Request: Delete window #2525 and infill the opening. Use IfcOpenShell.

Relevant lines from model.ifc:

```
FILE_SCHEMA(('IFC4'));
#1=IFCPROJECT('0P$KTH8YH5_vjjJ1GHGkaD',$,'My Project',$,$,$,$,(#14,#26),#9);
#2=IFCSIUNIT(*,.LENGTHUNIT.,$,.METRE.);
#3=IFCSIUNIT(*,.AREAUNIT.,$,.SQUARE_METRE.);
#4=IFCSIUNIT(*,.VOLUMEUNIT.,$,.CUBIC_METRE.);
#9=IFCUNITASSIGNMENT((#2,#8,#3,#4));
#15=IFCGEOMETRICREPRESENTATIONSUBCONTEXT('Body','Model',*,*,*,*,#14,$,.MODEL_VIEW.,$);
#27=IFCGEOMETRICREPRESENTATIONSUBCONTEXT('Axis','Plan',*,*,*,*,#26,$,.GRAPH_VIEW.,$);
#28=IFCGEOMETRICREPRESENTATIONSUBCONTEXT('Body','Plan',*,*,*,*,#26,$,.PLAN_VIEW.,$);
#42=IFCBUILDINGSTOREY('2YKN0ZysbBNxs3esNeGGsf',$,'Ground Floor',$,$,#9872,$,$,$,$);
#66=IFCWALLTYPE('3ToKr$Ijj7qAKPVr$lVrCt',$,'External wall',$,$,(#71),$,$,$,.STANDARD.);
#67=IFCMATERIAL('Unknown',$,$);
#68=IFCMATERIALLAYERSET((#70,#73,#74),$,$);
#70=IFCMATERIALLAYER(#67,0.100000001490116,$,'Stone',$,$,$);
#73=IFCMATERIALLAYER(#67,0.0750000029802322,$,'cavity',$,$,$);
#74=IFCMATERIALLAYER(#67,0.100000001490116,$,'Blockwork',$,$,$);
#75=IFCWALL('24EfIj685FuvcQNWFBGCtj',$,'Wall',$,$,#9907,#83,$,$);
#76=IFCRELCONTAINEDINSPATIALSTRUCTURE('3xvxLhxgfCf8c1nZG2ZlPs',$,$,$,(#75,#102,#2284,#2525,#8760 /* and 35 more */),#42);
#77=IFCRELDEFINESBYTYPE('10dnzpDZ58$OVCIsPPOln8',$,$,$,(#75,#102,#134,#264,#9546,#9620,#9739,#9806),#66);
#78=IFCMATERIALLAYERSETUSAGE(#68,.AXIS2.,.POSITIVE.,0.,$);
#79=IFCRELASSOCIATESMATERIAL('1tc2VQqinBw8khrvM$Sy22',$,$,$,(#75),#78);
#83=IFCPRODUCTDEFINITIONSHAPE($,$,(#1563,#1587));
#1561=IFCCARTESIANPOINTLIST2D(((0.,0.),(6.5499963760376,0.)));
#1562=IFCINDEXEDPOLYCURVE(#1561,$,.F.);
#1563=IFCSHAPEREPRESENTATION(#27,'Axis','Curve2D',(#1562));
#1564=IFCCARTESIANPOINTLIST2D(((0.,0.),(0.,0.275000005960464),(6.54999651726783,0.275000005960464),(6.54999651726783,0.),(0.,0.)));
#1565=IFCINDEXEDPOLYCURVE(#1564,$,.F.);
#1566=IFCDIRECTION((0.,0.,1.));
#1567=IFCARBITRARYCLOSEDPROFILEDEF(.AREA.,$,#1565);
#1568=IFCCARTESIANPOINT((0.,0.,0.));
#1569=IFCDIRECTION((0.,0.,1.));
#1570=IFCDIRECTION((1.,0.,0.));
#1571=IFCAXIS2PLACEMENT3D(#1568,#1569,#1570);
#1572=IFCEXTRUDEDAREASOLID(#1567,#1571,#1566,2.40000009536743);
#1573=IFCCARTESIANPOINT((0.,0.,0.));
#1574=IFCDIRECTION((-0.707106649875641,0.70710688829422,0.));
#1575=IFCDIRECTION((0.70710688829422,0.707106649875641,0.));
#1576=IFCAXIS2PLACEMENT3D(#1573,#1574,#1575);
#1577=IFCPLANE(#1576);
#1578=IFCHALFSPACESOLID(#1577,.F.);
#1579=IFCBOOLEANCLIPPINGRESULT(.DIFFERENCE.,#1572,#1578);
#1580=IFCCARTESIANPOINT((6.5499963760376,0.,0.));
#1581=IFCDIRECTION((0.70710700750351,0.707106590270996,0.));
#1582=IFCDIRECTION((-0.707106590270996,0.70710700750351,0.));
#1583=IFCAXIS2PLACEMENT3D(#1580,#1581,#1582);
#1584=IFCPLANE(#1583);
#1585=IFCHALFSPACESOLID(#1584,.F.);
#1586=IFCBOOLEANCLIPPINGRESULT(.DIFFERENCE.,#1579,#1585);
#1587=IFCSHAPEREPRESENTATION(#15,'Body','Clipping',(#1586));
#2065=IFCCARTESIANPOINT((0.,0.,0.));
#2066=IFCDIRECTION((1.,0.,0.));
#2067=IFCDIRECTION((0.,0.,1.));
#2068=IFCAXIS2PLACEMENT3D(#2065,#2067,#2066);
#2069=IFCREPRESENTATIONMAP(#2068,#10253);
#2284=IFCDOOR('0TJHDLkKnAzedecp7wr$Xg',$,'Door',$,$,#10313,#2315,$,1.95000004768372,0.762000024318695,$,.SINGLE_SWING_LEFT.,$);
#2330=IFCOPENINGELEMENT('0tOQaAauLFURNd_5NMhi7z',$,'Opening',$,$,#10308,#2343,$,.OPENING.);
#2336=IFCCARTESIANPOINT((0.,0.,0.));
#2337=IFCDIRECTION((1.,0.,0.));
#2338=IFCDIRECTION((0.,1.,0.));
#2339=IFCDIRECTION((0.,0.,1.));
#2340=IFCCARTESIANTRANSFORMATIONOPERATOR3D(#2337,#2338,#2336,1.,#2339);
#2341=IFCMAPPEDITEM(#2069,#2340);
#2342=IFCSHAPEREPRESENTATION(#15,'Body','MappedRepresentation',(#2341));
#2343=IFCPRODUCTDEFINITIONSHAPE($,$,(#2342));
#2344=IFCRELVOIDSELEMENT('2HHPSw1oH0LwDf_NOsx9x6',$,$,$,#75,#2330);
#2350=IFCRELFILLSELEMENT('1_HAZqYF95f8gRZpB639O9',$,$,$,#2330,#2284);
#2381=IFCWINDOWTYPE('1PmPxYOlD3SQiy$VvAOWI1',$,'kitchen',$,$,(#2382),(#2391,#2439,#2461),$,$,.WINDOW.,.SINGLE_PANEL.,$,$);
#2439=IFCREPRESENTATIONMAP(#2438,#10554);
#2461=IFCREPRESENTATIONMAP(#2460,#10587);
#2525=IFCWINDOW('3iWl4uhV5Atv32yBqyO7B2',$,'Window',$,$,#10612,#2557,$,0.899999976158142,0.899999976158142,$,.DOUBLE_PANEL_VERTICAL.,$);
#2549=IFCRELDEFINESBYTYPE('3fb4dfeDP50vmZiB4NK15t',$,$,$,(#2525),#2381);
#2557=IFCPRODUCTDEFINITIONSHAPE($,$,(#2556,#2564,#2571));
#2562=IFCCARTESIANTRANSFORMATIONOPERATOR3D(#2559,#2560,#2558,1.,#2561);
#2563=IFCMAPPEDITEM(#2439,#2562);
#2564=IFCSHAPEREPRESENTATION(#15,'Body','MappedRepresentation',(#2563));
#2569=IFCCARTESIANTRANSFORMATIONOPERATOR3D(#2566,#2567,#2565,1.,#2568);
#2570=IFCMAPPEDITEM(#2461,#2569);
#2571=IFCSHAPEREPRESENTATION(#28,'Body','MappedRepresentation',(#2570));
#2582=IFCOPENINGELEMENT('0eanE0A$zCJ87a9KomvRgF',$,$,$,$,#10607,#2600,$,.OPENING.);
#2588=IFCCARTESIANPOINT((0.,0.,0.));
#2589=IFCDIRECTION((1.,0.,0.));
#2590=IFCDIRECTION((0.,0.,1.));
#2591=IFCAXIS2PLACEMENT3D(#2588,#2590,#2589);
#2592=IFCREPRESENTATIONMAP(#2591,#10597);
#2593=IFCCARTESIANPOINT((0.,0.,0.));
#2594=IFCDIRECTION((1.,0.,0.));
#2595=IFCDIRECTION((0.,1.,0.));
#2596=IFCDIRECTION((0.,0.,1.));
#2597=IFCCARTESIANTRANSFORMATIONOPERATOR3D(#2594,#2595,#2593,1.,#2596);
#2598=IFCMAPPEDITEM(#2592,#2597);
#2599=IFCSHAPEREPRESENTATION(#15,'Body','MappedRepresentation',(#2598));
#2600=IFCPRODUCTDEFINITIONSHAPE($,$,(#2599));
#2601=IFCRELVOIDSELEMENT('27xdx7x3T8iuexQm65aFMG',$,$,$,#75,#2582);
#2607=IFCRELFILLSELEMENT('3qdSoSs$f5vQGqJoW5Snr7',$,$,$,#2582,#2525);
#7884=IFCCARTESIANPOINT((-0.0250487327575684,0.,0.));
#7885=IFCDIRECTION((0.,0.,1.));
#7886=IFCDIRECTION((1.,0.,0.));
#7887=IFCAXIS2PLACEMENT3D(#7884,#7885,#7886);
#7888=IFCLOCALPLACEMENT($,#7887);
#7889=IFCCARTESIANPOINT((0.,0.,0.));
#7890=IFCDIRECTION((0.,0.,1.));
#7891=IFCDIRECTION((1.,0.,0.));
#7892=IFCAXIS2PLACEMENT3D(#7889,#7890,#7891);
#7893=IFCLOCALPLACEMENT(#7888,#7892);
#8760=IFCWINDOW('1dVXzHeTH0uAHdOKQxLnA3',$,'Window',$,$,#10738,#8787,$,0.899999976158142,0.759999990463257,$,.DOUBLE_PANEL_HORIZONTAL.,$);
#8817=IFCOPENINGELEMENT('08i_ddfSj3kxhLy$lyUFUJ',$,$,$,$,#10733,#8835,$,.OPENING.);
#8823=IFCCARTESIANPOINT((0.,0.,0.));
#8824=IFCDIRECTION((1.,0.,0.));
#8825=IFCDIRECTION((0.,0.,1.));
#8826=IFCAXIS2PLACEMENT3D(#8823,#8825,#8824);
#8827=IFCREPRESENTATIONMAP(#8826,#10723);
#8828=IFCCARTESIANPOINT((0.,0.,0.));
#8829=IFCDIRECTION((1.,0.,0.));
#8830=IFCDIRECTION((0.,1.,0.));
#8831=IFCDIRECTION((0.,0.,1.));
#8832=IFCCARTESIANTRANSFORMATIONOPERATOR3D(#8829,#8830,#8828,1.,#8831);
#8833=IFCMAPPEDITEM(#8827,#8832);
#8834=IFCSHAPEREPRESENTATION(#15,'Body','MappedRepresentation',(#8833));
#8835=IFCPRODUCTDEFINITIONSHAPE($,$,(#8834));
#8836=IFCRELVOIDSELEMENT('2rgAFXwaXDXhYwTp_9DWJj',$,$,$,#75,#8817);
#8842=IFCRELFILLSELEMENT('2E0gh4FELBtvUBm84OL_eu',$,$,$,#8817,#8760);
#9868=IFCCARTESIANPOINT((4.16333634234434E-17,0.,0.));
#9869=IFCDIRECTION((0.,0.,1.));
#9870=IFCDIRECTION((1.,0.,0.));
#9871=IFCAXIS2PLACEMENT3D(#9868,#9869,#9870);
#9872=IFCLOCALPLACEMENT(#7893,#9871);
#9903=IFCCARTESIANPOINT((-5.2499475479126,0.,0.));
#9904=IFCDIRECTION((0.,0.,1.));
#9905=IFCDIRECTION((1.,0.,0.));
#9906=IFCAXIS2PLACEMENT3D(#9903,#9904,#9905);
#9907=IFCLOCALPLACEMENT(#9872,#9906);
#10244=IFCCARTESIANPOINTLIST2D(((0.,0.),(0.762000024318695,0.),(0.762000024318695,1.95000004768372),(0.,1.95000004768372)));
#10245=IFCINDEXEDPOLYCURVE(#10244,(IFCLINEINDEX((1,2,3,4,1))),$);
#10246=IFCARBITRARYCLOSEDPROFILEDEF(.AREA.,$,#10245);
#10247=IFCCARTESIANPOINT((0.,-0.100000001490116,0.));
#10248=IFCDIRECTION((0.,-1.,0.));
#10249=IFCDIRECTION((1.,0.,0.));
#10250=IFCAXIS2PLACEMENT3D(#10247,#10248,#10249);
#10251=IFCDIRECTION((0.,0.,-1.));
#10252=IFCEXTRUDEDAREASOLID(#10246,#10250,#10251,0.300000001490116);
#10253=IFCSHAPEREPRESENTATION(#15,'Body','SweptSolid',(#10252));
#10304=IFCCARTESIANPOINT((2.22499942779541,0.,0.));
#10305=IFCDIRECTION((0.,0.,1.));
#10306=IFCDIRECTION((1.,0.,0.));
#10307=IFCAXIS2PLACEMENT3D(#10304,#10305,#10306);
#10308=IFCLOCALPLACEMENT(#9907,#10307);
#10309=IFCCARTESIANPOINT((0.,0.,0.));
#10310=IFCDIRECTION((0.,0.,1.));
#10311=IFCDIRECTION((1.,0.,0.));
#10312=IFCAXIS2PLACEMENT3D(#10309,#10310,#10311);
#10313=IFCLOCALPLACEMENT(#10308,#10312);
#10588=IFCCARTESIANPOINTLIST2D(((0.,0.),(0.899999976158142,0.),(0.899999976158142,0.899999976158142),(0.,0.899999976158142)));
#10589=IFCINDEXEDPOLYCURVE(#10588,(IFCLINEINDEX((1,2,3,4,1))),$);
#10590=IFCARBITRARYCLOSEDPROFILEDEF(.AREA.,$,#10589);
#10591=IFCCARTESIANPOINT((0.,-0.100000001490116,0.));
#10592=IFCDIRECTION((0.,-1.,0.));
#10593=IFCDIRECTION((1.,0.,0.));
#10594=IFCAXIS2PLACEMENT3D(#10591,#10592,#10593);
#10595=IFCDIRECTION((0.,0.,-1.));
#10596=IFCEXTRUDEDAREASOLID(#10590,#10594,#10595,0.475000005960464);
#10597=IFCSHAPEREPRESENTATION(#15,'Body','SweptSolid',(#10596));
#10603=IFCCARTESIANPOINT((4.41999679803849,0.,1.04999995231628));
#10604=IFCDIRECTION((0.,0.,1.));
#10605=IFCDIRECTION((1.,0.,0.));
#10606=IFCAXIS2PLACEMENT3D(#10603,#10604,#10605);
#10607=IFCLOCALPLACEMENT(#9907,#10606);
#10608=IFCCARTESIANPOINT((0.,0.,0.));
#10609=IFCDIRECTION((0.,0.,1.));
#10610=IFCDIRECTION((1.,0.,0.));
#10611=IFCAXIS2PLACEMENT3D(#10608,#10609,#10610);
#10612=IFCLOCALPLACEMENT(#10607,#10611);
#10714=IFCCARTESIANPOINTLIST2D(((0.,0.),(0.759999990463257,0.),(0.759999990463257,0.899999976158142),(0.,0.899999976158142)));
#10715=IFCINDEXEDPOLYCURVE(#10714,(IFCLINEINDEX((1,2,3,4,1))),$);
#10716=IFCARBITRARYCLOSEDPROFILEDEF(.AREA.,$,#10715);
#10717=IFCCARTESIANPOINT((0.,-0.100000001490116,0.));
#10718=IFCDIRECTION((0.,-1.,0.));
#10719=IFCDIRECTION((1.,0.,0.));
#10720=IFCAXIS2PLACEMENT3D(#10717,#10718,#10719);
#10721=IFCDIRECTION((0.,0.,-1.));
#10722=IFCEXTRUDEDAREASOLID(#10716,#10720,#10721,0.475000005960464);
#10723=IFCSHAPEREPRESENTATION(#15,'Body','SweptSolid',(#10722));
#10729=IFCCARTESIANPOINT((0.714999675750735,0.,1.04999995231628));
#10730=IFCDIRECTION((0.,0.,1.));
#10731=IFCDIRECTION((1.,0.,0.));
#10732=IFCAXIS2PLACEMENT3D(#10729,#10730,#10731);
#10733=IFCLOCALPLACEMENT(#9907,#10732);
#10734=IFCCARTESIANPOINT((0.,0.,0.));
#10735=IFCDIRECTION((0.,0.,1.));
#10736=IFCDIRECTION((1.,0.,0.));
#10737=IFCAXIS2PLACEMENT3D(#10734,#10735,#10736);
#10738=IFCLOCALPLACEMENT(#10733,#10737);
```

```python
import ifcopenshell
import ifcopenshell.api.feature
import ifcopenshell.api.root
import ifcopenshell.geom
import ifcopenshell.util.shape

model = ifcopenshell.open("model.ifc")
settings = ifcopenshell.geom.settings()


def volume(element):
    """Net volume in cubic metres, openings subtracted."""
    shape = ifcopenshell.geom.create_shape(settings, element)
    return ifcopenshell.util.shape.get_volume(shape.geometry)


window = model.by_guid("3iWl4uhV5Atv32yBqyO7B2")
opening = window.FillsVoids[0].RelatingOpeningElement
wall = opening.VoidsElements[0].RelatingBuildingElement
before = volume(wall)

ifcopenshell.api.root.remove_product(model, product=window)
ifcopenshell.api.feature.remove_feature(model, feature=opening)

after = volume(wall)

print(f"wall volume {before:.3f} -> {after:.3f} m3")

model.write("model_v2.ifc")
```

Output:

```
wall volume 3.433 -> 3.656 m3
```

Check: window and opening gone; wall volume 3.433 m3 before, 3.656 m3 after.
